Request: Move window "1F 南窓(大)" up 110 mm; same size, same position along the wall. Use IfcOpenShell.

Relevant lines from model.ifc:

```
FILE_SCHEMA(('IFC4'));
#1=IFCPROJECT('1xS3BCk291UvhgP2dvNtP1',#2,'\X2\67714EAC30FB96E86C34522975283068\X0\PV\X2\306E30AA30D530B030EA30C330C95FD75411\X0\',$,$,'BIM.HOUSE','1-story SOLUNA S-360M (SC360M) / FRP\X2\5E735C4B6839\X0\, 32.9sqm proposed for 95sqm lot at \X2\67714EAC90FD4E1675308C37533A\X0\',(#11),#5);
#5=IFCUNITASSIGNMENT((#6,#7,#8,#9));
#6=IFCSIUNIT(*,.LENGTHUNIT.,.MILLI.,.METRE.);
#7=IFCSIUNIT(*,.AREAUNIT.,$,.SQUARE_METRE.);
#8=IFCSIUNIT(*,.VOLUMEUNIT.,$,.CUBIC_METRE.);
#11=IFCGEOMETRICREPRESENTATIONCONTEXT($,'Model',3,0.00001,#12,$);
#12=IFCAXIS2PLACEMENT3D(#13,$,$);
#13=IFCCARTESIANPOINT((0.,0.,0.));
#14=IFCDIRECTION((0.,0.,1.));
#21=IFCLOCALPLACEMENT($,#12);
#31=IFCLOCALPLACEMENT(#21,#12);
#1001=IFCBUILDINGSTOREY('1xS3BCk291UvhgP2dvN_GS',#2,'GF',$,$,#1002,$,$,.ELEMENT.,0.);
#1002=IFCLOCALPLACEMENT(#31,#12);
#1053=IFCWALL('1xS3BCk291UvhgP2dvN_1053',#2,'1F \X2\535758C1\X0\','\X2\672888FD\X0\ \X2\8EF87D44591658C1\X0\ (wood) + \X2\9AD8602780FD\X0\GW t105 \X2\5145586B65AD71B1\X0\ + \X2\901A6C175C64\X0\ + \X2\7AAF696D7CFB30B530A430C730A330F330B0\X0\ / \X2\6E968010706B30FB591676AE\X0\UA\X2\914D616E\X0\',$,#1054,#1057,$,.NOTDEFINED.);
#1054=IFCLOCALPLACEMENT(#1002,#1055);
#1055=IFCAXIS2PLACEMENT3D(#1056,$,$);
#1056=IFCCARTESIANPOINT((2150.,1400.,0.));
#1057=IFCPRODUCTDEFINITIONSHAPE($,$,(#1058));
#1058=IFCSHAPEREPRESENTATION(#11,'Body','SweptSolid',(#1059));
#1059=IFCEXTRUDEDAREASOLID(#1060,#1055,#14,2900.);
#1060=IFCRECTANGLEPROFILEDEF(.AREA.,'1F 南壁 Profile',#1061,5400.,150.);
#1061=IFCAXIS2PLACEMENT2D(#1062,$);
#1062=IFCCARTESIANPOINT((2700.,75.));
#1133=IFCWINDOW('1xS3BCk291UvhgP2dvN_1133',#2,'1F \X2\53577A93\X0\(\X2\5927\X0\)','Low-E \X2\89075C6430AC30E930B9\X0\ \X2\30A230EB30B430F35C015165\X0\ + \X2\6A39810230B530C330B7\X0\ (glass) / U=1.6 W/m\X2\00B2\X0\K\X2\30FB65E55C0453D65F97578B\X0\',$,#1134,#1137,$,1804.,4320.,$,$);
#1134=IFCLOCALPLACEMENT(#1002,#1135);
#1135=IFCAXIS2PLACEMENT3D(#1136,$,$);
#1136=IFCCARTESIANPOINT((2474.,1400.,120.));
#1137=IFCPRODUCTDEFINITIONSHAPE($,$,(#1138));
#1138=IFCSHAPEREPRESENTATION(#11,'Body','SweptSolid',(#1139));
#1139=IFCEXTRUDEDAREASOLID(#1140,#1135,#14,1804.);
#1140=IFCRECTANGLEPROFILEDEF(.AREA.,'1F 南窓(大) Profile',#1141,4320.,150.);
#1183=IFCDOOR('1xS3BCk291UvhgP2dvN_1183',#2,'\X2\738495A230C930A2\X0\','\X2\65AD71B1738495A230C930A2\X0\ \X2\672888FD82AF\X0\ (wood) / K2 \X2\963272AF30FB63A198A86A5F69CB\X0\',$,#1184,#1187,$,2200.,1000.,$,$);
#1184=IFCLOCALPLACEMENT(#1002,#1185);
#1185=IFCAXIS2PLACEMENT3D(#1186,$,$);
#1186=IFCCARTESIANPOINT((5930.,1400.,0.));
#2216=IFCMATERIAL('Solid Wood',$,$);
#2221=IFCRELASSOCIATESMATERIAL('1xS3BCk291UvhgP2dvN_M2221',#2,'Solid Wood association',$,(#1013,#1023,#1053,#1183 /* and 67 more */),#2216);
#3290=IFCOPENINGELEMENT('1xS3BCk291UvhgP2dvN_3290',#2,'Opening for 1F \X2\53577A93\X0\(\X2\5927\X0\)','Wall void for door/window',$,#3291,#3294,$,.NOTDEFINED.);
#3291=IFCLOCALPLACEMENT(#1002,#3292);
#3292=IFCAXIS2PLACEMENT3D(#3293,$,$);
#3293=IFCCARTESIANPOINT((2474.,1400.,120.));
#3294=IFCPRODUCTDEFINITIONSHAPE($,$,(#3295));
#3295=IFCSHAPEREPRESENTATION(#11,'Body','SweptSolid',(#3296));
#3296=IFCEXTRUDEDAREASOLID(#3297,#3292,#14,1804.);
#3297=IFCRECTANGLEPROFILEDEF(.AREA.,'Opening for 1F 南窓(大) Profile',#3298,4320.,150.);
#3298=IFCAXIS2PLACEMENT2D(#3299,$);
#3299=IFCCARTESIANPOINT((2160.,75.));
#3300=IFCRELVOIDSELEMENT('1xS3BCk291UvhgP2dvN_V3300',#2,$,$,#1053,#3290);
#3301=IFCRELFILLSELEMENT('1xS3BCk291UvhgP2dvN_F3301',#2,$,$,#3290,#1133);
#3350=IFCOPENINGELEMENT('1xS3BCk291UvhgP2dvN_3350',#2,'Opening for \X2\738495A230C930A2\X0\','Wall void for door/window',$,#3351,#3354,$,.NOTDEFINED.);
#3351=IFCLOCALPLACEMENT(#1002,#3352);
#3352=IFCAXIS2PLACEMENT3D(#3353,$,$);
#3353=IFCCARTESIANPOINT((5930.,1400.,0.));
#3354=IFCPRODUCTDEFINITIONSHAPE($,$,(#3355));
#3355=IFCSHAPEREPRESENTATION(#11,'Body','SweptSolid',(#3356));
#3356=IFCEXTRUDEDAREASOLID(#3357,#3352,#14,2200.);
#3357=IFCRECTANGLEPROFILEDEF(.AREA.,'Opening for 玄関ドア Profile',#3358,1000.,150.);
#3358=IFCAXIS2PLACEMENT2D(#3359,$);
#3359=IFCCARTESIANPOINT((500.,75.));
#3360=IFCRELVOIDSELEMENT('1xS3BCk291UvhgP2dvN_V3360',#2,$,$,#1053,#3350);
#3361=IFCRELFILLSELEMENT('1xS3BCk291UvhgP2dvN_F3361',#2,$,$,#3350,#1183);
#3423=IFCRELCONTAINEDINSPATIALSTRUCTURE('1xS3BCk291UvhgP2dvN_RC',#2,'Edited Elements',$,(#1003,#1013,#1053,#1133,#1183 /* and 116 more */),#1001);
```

```python
import numpy as np
import ifcopenshell
import ifcopenshell.api.geometry
import ifcopenshell.util.placement
import ifcopenshell.util.unit

model = ifcopenshell.open("model.ifc")
unit_scale = ifcopenshell.util.unit.calculate_unit_scale(model)

window = model.by_id(1133)
opening = window.FillsVoids[0].RelatingOpeningElement
dz = 0.11 / unit_scale

shift = np.array([0.0, 0.0, dz])
# The window is not placed relative to its opening, so move both.
for product in (opening, window):
    matrix = ifcopenshell.util.placement.get_local_placement(product.ObjectPlacement)
    matrix[:3, 3] += shift
    ifcopenshell.api.geometry.edit_object_placement(model, product=product, matrix=matrix, is_si=False)

print(f"moved by {dz * unit_scale:+.3f} m")

model.write("model_updated.ifc")
```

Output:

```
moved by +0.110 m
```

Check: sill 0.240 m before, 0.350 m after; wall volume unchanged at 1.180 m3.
